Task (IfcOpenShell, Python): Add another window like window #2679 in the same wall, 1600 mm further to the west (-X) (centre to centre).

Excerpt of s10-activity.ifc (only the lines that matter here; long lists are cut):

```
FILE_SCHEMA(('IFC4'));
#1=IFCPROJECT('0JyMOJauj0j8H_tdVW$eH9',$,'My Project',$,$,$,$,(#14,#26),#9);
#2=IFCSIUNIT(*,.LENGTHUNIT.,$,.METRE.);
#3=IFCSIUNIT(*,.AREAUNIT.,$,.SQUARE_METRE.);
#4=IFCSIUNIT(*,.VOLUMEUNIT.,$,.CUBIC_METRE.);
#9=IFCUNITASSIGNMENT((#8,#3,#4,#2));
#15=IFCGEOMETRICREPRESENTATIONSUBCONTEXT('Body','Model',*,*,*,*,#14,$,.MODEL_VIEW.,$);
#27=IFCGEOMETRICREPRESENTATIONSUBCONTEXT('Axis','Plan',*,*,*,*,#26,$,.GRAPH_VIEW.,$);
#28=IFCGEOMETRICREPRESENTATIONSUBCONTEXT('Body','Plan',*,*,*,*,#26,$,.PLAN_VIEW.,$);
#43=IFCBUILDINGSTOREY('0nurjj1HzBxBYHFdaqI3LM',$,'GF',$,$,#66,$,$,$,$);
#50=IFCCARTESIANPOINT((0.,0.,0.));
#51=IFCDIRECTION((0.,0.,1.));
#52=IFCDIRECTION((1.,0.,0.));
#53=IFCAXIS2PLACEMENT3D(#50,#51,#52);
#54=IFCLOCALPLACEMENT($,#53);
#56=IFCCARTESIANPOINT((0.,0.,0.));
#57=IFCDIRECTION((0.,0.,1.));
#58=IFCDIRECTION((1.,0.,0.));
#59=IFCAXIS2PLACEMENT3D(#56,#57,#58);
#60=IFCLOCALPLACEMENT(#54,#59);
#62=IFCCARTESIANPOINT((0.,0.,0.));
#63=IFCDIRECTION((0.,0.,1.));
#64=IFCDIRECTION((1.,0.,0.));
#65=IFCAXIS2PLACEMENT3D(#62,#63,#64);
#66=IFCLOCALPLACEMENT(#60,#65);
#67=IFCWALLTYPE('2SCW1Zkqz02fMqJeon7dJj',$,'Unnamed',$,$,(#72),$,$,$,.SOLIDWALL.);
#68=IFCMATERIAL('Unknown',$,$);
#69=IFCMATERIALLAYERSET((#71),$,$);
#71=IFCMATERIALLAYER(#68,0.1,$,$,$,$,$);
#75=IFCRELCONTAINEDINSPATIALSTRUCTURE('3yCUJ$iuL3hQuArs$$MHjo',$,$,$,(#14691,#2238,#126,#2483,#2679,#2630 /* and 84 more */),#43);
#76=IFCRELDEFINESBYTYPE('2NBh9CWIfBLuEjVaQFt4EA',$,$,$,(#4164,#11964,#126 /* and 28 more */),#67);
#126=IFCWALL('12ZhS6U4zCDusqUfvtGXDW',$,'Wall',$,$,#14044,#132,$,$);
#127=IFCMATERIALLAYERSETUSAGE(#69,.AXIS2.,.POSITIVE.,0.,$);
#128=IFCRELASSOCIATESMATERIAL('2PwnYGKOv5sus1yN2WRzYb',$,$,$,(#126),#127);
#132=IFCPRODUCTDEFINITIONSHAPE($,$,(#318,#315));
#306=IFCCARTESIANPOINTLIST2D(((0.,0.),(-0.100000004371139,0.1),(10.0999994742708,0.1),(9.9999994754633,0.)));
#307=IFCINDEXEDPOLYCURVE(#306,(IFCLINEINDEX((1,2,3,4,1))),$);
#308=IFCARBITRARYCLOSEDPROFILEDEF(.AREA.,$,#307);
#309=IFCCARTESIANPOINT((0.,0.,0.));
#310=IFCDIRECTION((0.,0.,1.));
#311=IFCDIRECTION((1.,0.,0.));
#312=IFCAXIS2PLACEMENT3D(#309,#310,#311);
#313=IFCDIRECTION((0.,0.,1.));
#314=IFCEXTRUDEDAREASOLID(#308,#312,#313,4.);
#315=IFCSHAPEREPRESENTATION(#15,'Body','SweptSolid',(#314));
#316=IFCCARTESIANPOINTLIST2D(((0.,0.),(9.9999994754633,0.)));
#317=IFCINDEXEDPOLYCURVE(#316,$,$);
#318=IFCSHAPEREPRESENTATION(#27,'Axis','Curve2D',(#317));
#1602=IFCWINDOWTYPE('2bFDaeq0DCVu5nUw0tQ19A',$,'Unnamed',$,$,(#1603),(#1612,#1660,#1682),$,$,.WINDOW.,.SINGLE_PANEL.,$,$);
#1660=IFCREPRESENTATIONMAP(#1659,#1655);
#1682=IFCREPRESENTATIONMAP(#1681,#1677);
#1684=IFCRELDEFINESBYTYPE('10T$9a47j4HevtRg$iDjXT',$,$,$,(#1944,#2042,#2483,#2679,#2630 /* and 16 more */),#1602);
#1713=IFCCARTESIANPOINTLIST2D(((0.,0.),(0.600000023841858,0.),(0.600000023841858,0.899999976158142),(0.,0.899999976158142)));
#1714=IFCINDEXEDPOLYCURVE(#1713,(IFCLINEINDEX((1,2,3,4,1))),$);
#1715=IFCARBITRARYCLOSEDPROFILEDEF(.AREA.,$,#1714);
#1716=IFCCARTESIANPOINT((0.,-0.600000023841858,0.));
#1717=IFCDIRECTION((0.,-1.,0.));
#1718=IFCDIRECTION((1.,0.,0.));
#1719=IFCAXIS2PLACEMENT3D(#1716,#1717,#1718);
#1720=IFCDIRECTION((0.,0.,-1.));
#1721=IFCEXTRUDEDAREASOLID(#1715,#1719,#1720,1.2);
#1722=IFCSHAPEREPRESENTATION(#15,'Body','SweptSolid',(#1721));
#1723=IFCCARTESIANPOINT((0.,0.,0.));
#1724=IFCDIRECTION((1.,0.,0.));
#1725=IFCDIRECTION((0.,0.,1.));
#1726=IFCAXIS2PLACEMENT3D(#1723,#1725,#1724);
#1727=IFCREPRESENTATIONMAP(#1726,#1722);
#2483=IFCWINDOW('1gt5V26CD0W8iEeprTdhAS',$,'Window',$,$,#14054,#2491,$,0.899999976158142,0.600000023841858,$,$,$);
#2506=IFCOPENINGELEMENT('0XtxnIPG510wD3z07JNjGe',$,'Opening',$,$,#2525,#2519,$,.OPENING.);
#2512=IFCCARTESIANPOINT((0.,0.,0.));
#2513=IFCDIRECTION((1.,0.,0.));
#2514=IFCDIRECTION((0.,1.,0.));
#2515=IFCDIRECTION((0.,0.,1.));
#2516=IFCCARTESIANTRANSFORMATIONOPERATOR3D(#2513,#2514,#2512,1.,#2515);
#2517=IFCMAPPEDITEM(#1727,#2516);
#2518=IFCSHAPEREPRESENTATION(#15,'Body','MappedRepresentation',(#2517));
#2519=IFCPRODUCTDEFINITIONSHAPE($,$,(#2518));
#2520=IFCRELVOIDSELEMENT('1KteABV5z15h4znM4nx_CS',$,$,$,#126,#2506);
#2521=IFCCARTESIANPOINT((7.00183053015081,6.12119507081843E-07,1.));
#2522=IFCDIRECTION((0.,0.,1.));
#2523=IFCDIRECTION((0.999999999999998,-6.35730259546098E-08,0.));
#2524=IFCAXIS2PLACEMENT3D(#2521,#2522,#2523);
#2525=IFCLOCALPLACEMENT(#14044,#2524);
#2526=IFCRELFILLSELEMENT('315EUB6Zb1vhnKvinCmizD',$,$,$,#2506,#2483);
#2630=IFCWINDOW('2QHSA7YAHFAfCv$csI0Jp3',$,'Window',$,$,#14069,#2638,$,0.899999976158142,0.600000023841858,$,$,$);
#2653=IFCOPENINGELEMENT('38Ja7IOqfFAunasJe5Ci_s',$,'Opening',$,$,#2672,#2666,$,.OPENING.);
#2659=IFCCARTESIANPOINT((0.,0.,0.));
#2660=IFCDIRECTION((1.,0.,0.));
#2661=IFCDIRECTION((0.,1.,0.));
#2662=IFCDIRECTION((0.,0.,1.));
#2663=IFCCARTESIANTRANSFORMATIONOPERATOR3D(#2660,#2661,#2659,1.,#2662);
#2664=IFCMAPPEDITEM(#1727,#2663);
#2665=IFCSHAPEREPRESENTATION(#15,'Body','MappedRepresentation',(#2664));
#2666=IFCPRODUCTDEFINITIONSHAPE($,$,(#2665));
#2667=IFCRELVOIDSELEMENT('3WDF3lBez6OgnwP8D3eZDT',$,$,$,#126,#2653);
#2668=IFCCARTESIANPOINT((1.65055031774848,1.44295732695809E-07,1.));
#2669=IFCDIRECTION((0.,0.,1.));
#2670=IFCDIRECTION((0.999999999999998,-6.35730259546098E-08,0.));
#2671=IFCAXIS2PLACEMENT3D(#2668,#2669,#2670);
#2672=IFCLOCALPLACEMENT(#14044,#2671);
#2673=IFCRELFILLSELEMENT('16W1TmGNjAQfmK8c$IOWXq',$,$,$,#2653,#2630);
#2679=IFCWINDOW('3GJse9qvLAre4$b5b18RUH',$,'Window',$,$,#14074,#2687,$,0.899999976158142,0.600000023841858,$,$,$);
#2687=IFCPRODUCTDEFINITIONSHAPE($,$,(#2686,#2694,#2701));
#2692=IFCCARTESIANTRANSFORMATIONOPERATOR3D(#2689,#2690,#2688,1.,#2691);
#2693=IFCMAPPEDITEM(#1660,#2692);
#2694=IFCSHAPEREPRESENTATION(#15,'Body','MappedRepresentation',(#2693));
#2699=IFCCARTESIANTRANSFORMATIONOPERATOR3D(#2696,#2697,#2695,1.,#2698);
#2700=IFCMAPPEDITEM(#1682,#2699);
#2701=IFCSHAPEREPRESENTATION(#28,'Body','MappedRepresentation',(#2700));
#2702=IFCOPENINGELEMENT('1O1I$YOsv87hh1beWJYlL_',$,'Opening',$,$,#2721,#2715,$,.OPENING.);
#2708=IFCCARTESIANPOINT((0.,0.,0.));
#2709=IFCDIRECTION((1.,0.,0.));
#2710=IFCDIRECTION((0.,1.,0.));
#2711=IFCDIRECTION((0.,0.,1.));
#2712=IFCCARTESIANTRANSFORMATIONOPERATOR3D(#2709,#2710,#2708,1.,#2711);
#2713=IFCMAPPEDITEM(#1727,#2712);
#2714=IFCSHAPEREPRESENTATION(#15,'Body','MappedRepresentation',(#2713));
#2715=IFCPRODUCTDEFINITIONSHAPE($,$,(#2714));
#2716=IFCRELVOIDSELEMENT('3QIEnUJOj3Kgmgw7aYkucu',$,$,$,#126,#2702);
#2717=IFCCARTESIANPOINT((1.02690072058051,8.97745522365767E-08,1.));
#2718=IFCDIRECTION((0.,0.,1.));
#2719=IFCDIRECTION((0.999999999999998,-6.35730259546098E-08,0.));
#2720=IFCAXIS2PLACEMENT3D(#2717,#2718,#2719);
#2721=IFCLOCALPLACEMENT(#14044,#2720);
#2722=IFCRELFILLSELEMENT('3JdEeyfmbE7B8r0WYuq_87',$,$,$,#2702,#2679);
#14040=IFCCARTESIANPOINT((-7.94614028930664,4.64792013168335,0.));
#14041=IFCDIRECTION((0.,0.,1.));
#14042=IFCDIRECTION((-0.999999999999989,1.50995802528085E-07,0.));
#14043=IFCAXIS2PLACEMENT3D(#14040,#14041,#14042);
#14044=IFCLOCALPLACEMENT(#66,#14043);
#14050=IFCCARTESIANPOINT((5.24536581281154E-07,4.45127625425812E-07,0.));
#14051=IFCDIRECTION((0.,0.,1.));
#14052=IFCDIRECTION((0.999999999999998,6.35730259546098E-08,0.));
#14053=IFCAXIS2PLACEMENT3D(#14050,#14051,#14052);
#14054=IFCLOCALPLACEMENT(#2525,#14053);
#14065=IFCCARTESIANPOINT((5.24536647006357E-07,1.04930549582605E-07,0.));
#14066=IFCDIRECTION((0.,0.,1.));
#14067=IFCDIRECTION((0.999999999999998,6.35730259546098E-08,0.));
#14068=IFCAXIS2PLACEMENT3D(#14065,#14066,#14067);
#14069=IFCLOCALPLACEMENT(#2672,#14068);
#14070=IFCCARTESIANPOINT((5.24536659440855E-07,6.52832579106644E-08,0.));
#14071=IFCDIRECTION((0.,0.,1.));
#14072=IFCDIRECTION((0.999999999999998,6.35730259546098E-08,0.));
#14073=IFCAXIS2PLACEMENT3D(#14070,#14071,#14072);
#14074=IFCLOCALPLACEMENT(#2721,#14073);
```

```python
import ifcopenshell
import ifcopenshell.api.feature
import ifcopenshell.api.geometry
import ifcopenshell.api.root
import ifcopenshell.geom
import ifcopenshell.util.element
import ifcopenshell.util.placement
import ifcopenshell.util.shape
import ifcopenshell.util.unit

model = ifcopenshell.open("s10-activity.ifc")
unit_scale = ifcopenshell.util.unit.calculate_unit_scale(model)
settings = ifcopenshell.geom.settings()


def volume(element):
    """Net volume in cubic metres, openings subtracted."""
    shape = ifcopenshell.geom.create_shape(settings, element)
    return ifcopenshell.util.shape.get_volume(shape.geometry)


window = model.by_guid("3GJse9qvLAre4$b5b18RUH")
opening = window.FillsVoids[0].RelatingOpeningElement
wall = opening.VoidsElements[0].RelatingBuildingElement
before = volume(wall)
shift = ifcopenshell.util.placement.get_local_placement(wall.ObjectPlacement)[:3, 0] * 1.6 / unit_scale

# copy_class copies the void relationship, type, container and properties, but no geometry.
new_opening = ifcopenshell.api.root.copy_class(model, product=opening)
new_opening.Representation = ifcopenshell.util.element.copy_deep(
    model, opening.Representation, exclude=["IfcGeometricRepresentationContext", "IfcRepresentationMap"]
)
new_window = ifcopenshell.api.root.copy_class(model, product=window)
new_window.Representation = ifcopenshell.util.element.copy_deep(
    model, window.Representation, exclude=["IfcGeometricRepresentationContext", "IfcRepresentationMap"]
)
ifcopenshell.api.feature.add_filling(model, opening=new_opening, element=new_window)

for old, new in ((opening, new_opening), (window, new_window)):
    matrix = ifcopenshell.util.placement.get_local_placement(old.ObjectPlacement)
    matrix[:3, 3] += shift
    ifcopenshell.api.geometry.edit_object_placement(model, product=new, matrix=matrix, is_si=False)

after = volume(wall)

print(f"wall volume {before:.3f} -> {after:.3f} m3")

model.write("s10-activity_updated.ifc")
```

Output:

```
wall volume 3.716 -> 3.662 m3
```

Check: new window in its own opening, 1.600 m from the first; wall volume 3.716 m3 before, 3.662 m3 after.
